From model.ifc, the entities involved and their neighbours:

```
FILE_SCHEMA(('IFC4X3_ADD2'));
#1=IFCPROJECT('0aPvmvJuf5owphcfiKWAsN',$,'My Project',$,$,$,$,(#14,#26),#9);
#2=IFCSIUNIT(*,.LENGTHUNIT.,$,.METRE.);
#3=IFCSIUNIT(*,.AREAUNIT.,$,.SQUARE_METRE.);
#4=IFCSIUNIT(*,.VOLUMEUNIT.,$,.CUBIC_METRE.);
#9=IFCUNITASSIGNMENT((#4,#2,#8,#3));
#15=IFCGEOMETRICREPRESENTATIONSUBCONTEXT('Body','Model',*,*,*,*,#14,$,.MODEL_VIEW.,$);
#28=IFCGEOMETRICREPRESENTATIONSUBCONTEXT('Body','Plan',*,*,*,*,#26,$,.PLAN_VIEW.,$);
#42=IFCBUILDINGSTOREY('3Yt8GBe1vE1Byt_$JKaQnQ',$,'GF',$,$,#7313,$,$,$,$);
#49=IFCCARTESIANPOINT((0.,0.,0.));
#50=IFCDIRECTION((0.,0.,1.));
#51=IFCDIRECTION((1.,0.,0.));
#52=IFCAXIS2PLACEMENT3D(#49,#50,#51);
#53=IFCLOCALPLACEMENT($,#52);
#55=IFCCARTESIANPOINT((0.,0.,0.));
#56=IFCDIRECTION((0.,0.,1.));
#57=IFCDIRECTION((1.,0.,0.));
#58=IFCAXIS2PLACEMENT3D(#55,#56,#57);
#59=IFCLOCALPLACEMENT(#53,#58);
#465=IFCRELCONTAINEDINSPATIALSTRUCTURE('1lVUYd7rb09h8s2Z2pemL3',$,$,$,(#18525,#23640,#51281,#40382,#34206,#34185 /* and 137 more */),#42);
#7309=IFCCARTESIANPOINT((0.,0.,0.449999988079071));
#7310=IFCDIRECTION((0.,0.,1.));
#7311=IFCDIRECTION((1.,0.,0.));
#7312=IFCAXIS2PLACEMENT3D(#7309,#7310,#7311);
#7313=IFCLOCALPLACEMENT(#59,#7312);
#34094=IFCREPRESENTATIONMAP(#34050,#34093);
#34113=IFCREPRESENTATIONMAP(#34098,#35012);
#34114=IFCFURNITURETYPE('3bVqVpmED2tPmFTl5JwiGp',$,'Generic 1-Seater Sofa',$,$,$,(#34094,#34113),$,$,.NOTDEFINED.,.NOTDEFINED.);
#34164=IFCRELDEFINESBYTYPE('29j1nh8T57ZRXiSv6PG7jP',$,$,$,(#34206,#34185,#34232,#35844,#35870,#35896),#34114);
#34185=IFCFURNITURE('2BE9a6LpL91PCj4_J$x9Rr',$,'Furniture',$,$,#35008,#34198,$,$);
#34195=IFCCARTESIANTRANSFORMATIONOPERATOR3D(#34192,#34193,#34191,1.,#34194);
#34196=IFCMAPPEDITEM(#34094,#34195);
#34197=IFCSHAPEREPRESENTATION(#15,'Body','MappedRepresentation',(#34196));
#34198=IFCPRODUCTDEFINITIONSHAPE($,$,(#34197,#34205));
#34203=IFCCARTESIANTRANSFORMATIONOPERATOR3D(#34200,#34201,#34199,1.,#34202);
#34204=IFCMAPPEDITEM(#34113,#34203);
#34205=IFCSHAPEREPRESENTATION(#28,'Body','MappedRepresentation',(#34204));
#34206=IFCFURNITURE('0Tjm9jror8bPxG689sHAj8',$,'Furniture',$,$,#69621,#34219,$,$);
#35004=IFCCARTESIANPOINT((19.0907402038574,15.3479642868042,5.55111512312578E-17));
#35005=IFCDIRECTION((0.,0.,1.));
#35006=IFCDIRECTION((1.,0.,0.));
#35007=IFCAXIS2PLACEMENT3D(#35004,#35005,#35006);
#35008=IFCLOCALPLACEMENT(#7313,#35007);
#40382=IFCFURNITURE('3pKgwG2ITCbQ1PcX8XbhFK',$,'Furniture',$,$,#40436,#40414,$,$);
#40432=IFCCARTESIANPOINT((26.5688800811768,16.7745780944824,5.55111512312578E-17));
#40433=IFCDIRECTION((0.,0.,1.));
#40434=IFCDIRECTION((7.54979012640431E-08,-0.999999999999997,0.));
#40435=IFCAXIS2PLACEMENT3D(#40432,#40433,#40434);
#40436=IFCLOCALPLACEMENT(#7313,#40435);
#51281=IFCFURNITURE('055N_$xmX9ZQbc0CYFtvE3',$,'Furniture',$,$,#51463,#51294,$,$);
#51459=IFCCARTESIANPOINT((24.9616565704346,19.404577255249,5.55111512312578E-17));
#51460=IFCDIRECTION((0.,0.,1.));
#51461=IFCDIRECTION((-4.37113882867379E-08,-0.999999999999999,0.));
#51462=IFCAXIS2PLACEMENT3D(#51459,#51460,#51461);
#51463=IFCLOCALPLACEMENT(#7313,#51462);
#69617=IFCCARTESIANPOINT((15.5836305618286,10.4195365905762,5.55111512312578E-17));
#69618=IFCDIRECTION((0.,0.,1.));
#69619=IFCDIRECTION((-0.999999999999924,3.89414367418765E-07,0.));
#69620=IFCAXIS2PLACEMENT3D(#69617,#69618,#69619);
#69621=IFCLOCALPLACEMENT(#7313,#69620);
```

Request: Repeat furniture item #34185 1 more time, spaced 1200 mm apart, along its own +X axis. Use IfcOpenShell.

```python
import ifcopenshell
import ifcopenshell.api.geometry
import ifcopenshell.api.root
import ifcopenshell.util.element
import ifcopenshell.util.placement

model = ifcopenshell.open("model.ifc")

source = model.by_id(34185)
base = ifcopenshell.util.placement.get_local_placement(source.ObjectPlacement)
step = base[:3, 0] * 1.2

for i in range(1, 2):
    copy = ifcopenshell.api.root.copy_class(model, product=source)
    copy.Representation = ifcopenshell.util.element.copy_deep(
        model, source.Representation, exclude=["IfcGeometricRepresentationContext", "IfcRepresentationMap"]
    )
    matrix = base.copy()
    matrix[:3, 3] += i * step
    print("added at", matrix[:3, 3].round(3) + 0.0)
    ifcopenshell.api.geometry.edit_object_placement(model, product=copy, matrix=matrix, is_si=False)

model.write("model_v2.ifc")
```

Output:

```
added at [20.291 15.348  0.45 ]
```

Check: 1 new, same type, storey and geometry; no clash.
